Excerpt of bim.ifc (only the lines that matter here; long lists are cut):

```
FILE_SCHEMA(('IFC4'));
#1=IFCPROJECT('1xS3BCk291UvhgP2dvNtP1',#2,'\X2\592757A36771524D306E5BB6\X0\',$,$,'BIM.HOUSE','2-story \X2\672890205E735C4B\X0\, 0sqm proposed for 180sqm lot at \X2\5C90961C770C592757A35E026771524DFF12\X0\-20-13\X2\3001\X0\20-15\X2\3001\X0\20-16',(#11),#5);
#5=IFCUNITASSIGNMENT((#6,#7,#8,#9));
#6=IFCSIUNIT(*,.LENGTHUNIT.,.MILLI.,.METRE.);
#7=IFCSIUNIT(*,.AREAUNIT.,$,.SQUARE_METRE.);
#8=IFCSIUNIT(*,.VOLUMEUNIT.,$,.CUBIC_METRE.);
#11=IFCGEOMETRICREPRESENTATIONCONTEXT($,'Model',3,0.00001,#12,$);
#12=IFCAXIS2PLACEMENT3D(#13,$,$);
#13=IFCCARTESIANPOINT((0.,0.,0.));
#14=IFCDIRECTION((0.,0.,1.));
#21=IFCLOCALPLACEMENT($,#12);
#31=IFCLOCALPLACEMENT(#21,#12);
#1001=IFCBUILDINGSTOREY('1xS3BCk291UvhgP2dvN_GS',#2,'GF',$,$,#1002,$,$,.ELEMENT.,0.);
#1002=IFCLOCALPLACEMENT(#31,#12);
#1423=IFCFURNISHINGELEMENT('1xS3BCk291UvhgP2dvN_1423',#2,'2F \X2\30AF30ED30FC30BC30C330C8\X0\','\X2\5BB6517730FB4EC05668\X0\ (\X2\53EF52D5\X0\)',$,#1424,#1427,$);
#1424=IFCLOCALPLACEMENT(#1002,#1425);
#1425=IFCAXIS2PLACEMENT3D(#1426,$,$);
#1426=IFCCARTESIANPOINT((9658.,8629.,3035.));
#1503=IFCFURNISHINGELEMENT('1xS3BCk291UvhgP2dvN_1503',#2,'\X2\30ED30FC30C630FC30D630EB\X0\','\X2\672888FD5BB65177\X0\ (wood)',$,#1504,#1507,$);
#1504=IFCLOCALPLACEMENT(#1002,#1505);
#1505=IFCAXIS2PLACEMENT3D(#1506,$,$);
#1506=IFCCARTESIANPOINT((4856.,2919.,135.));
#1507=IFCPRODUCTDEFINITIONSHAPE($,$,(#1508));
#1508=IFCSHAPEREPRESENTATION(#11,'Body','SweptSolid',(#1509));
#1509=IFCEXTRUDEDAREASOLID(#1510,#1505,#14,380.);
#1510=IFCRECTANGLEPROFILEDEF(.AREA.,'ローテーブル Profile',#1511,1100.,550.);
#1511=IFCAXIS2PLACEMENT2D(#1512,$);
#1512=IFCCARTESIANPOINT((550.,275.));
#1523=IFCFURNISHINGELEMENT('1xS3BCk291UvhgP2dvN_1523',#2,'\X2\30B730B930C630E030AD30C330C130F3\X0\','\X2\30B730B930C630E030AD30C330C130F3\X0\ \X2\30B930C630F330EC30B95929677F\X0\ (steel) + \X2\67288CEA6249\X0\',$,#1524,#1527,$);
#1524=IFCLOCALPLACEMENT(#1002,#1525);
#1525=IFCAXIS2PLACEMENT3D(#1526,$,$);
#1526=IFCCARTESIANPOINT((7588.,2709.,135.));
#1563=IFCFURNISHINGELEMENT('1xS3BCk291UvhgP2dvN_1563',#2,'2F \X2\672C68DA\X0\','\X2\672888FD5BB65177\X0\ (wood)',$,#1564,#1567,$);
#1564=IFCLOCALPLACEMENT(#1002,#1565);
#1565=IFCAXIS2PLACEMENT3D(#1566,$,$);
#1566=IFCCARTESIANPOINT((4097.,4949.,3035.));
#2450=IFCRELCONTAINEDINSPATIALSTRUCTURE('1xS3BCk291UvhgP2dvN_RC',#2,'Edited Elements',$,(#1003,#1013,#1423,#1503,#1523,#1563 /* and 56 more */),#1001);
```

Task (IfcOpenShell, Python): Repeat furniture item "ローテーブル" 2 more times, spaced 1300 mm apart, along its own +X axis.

```python
import ifcopenshell
import ifcopenshell.api.geometry
import ifcopenshell.api.root
import ifcopenshell.util.element
import ifcopenshell.util.placement
import ifcopenshell.util.unit

model = ifcopenshell.open("bim.ifc")
unit_scale = ifcopenshell.util.unit.calculate_unit_scale(model)


def reuse_history(source, copy):
    """copy_class also copies each property set's owner history, people and application; keep the originals."""
    for rel in copy.IsDefinedBy:
        if rel.is_a("IfcRelDefinesByProperties") and (history := rel.RelatingPropertyDefinition.OwnerHistory):
            rel.RelatingPropertyDefinition.OwnerHistory = source.OwnerHistory
            ifcopenshell.util.element.remove_deep2(model, history)


source = model.by_id(1503)
base = ifcopenshell.util.placement.get_local_placement(source.ObjectPlacement)
step = base[:3, 0] * 1.3 / unit_scale

for i in range(1, 3):
    copy = ifcopenshell.api.root.copy_class(model, product=source)
    copy.Representation = ifcopenshell.util.element.copy_deep(
        model, source.Representation, exclude=["IfcGeometricRepresentationContext", "IfcRepresentationMap"]
    )
    reuse_history(source, copy)
    matrix = base.copy()
    matrix[:3, 3] += i * step
    print("added at", matrix[:3, 3].round(3) + 0.0)
    ifcopenshell.api.geometry.edit_object_placement(model, product=copy, matrix=matrix, is_si=False)

model.write("bim_rev.ifc")
```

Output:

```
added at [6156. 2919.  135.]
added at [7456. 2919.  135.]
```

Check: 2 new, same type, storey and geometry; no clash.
